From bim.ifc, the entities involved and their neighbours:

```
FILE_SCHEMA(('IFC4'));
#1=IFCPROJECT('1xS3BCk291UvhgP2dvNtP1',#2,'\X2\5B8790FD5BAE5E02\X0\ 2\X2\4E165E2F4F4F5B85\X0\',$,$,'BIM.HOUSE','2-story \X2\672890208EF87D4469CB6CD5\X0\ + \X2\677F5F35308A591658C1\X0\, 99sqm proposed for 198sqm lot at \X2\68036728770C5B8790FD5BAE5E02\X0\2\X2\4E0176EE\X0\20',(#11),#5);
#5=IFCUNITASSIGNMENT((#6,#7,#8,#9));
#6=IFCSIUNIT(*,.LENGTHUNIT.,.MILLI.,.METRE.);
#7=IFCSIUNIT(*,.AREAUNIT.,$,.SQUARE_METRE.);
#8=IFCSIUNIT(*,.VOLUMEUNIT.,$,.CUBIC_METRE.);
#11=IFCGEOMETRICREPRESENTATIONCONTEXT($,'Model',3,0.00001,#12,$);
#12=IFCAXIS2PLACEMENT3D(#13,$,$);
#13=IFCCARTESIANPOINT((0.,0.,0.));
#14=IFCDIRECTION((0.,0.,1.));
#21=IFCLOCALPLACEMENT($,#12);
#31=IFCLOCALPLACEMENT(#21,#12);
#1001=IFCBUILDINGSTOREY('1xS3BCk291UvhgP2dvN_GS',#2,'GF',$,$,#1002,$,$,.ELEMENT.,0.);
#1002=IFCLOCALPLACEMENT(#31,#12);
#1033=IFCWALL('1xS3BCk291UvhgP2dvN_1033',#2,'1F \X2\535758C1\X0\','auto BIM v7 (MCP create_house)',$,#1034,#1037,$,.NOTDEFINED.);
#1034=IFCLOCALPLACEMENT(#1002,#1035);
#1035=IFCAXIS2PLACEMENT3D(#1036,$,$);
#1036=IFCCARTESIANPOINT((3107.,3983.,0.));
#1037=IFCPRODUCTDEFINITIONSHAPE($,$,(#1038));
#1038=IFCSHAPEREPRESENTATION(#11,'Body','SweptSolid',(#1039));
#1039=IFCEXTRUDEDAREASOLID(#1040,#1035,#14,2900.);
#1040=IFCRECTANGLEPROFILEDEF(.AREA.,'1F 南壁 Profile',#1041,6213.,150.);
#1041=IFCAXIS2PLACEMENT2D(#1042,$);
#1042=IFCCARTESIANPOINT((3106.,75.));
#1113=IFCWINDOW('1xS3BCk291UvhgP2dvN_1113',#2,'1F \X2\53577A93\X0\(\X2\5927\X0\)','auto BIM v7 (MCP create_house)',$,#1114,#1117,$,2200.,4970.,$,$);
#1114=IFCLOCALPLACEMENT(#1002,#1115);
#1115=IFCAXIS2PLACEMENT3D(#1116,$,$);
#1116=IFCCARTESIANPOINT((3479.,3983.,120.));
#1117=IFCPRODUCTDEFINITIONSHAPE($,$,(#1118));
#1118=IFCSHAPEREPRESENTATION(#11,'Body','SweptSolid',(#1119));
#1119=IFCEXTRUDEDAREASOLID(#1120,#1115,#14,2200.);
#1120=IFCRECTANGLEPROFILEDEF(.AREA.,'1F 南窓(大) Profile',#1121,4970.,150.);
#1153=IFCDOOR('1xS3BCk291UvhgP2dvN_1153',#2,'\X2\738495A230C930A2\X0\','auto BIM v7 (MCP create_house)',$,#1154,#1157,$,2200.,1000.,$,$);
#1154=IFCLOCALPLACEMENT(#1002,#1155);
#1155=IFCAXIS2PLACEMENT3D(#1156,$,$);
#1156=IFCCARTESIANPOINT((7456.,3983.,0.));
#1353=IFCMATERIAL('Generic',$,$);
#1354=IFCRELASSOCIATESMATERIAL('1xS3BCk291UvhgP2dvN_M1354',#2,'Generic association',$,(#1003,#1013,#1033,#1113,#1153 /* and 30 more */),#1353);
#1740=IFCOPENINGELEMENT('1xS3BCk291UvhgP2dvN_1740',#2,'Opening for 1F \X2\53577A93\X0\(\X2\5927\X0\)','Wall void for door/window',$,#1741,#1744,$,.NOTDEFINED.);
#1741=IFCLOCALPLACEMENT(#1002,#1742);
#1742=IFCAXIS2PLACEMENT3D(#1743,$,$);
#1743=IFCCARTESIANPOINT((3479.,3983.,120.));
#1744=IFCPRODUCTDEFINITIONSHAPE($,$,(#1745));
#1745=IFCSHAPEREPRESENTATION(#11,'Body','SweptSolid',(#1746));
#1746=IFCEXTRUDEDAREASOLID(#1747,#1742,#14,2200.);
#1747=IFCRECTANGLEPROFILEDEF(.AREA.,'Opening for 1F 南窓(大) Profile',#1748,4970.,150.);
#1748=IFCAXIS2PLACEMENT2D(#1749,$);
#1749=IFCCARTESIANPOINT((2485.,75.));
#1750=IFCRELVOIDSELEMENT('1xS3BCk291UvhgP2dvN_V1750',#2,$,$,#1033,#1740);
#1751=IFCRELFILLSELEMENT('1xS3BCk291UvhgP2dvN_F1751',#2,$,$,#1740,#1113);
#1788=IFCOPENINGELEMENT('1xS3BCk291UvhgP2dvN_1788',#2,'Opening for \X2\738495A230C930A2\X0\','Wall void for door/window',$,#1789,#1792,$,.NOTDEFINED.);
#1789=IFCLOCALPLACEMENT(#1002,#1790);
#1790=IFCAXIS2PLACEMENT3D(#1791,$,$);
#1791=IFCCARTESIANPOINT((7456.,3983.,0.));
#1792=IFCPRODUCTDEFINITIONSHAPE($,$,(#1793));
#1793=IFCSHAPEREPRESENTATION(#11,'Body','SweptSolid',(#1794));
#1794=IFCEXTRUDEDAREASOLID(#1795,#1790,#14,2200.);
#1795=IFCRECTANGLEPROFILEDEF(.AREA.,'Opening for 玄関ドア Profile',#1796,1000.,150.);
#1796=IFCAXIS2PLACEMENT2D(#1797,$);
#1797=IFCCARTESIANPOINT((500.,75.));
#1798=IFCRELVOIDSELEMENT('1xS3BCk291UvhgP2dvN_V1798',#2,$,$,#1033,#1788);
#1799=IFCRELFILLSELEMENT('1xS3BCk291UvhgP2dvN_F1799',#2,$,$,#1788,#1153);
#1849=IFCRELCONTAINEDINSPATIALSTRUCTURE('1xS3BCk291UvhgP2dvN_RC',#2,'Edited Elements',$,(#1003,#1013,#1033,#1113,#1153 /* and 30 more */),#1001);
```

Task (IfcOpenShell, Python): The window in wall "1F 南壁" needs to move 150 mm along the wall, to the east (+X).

```python
import ifcopenshell
import ifcopenshell.api.geometry
import ifcopenshell.util.placement
import ifcopenshell.util.unit

model = ifcopenshell.open("bim.ifc")
unit_scale = ifcopenshell.util.unit.calculate_unit_scale(model)

window = model.by_guid("1xS3BCk291UvhgP2dvN_1113")
opening = window.FillsVoids[0].RelatingOpeningElement
wall = opening.VoidsElements[0].RelatingBuildingElement

wall_matrix = ifcopenshell.util.placement.get_local_placement(wall.ObjectPlacement)
shift = wall_matrix[:3, 0] * 0.15 / unit_scale
before = ifcopenshell.util.placement.get_local_placement(window.ObjectPlacement)[:3, 3].copy()

# The window is not placed relative to its opening, so move both.
for product in (opening, window):
    matrix = ifcopenshell.util.placement.get_local_placement(product.ObjectPlacement)
    matrix[:3, 3] += shift
    ifcopenshell.api.geometry.edit_object_placement(model, product=product, matrix=matrix, is_si=False)

after = ifcopenshell.util.placement.get_local_placement(window.ObjectPlacement)[:3, 3]
print("window moved by", (after - before).round(3) + 0.0)

model.write("bim_edited.ifc")
```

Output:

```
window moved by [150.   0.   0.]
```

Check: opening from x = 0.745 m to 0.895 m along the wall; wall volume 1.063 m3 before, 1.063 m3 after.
